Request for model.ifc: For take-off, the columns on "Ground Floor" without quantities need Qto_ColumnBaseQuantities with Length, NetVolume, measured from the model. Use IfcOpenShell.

First a look at what the model holds.

```python
import ifcopenshell
import ifcopenshell.util.element
import ifcopenshell.util.unit

model = ifcopenshell.open("model.ifc")
print(model.schema)
for unit_type in ("LENGTHUNIT", "AREAUNIT", "VOLUMEUNIT"):
    print(unit_type, ifcopenshell.util.unit.calculate_unit_scale(model, unit_type))
storey = next(s for s in model.by_type("IfcBuildingStorey") if s.Name == "Ground Floor")
columns = [e for e in ifcopenshell.util.element.get_decomposition(storey) if e.is_a("IfcColumn")]
for e in sorted(columns, key=lambda e: e.id()):
    print(e.id(), e.is_a(), e.Name, list(ifcopenshell.util.element.get_psets(e, qtos_only=True)), sep=" | ")
```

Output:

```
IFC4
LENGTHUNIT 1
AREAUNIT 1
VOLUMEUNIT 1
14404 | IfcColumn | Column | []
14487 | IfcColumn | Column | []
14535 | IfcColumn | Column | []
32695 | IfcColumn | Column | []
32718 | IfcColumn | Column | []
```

```python
import ifcopenshell
import ifcopenshell.api.pset
import ifcopenshell.geom
import ifcopenshell.util.element
import ifcopenshell.util.shape
import ifcopenshell.util.unit

model = ifcopenshell.open("model.ifc")
unit_scale = ifcopenshell.util.unit.calculate_unit_scale(model)
volume_scale = ifcopenshell.util.unit.calculate_unit_scale(model, "VOLUMEUNIT")
settings = ifcopenshell.geom.settings()

storey = next(s for s in model.by_type("IfcBuildingStorey") if s.Name == "Ground Floor")
columns = [e for e in ifcopenshell.util.element.get_decomposition(storey) if e.is_a("IfcColumn")]

for e in sorted(columns, key=lambda e: e.id()):
    if ifcopenshell.util.element.get_psets(e, qtos_only=True, should_inherit=False):
        continue
    # Geometry comes back in metres, in the element's own axes.
    shape = ifcopenshell.geom.create_shape(settings, e)
    values = {
        "Length": ifcopenshell.util.shape.get_z(shape.geometry) / unit_scale,
        "NetVolume": ifcopenshell.util.shape.get_volume(shape.geometry) / volume_scale,
    }
    qto = ifcopenshell.api.pset.add_qto(model, product=e, name="Qto_ColumnBaseQuantities")
    ifcopenshell.api.pset.edit_qto(model, qto=qto, properties=values)
    print(e.id(), {k: round(v, 3) for k, v in values.items()})

model.write("model_updated.ifc")
```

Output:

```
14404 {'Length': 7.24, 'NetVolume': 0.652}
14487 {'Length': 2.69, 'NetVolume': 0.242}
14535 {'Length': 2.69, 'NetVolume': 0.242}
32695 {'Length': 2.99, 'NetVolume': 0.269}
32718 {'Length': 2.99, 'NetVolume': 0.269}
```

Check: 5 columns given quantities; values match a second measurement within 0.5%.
